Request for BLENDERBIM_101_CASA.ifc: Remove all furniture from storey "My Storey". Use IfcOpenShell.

First a look at what the model holds.

```python
import ifcopenshell
import ifcopenshell.util.element

model = ifcopenshell.open("BLENDERBIM_101_CASA.ifc")
print(model.schema)
storey = next(s for s in model.by_type("IfcBuildingStorey") if s.Name == "My Storey")
furniture = [e for e in ifcopenshell.util.element.get_decomposition(storey) if e.is_a("IfcFurnishingElement")]
seen = {}
for e in furniture:
    element_type = ifcopenshell.util.element.get_type(e)
    name = element_type.Name if element_type not in (None, e) else None
    seen[name] = seen.get(name, 0) + 1
for name, count in sorted(seen.items(), key=str):
    print(count, "x", name)
```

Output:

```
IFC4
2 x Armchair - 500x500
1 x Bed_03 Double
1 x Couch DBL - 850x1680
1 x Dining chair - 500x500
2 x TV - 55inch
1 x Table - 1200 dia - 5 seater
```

```python
import ifcopenshell
import ifcopenshell.api.root
import ifcopenshell.util.element

model = ifcopenshell.open("BLENDERBIM_101_CASA.ifc")

storey = next(s for s in model.by_type("IfcBuildingStorey") if s.Name == "My Storey")
furniture = [e for e in ifcopenshell.util.element.get_decomposition(storey) if e.is_a("IfcFurnishingElement")]

for e in furniture:
    ifcopenshell.api.root.remove_product(model, product=e)
print(len(furniture), "removed")

model.write("BLENDERBIM_101_CASA_edited.ifc")
```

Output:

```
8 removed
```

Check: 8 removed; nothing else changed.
